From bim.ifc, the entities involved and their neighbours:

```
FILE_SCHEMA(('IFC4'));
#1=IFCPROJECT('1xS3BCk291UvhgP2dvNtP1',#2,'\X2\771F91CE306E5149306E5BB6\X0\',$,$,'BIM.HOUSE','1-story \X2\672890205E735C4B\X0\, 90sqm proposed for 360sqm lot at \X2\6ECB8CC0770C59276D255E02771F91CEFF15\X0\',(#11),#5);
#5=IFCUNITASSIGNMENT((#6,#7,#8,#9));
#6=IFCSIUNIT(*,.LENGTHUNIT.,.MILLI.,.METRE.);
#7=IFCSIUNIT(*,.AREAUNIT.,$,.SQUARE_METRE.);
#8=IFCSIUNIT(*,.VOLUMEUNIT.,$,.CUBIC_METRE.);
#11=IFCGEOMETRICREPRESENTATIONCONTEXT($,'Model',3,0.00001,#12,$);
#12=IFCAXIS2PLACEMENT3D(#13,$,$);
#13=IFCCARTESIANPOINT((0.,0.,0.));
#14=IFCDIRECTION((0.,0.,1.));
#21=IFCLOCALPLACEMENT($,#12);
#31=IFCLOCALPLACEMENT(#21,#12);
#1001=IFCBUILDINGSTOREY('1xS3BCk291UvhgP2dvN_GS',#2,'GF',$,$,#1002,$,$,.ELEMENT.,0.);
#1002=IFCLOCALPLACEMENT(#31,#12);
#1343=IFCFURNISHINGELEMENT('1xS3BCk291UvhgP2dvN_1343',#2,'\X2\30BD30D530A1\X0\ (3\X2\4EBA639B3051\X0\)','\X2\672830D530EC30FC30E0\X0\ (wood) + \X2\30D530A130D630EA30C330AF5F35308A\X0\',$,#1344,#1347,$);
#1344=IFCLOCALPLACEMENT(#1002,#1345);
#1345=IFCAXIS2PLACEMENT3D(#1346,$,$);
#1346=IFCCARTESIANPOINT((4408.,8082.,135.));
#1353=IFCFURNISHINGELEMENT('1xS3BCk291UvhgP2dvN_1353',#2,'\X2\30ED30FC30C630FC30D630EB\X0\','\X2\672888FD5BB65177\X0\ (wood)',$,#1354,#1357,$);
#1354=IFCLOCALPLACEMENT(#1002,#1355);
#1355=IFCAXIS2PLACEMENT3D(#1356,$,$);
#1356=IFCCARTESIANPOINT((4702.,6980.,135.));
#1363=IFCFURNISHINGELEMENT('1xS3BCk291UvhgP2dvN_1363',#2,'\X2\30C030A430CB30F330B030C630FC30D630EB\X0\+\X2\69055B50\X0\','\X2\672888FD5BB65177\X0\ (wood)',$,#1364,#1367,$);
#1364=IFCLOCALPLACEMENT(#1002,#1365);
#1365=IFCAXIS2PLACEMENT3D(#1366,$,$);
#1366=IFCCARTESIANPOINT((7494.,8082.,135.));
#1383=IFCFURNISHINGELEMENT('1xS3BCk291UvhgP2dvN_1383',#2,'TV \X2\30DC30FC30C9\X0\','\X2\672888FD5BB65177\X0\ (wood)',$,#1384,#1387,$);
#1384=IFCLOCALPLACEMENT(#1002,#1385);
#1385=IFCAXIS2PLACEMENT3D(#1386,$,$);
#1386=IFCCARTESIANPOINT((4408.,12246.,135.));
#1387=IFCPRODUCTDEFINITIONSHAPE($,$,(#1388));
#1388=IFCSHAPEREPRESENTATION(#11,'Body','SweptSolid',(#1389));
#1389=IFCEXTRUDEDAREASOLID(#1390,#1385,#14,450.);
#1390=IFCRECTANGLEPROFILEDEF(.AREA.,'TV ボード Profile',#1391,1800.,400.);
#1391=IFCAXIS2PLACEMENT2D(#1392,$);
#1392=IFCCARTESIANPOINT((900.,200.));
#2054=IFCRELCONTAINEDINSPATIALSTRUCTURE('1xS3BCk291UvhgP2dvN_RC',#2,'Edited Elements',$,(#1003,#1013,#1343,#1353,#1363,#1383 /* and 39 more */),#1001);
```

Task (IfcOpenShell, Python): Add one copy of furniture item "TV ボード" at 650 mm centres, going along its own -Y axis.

```python
import ifcopenshell
import ifcopenshell.api.geometry
import ifcopenshell.api.root
import ifcopenshell.util.element
import ifcopenshell.util.placement
import ifcopenshell.util.unit

model = ifcopenshell.open("bim.ifc")
unit_scale = ifcopenshell.util.unit.calculate_unit_scale(model)


def reuse_history(source, copy):
    """copy_class also copies each property set's owner history, people and application; keep the originals."""
    for rel in copy.IsDefinedBy:
        if rel.is_a("IfcRelDefinesByProperties") and (history := rel.RelatingPropertyDefinition.OwnerHistory):
            rel.RelatingPropertyDefinition.OwnerHistory = source.OwnerHistory
            ifcopenshell.util.element.remove_deep2(model, history)


source = model.by_guid("1xS3BCk291UvhgP2dvN_1383")
base = ifcopenshell.util.placement.get_local_placement(source.ObjectPlacement)
step = -base[:3, 1] * 0.65 / unit_scale

for i in range(1, 2):
    copy = ifcopenshell.api.root.copy_class(model, product=source)
    copy.Representation = ifcopenshell.util.element.copy_deep(
        model, source.Representation, exclude=["IfcGeometricRepresentationContext", "IfcRepresentationMap"]
    )
    reuse_history(source, copy)
    matrix = base.copy()
    matrix[:3, 3] += i * step
    print("added at", matrix[:3, 3].round(3) + 0.0)
    ifcopenshell.api.geometry.edit_object_placement(model, product=copy, matrix=matrix, is_si=False)

model.write("bim_edited.ifc")
```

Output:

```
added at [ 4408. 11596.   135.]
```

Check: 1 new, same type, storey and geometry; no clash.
